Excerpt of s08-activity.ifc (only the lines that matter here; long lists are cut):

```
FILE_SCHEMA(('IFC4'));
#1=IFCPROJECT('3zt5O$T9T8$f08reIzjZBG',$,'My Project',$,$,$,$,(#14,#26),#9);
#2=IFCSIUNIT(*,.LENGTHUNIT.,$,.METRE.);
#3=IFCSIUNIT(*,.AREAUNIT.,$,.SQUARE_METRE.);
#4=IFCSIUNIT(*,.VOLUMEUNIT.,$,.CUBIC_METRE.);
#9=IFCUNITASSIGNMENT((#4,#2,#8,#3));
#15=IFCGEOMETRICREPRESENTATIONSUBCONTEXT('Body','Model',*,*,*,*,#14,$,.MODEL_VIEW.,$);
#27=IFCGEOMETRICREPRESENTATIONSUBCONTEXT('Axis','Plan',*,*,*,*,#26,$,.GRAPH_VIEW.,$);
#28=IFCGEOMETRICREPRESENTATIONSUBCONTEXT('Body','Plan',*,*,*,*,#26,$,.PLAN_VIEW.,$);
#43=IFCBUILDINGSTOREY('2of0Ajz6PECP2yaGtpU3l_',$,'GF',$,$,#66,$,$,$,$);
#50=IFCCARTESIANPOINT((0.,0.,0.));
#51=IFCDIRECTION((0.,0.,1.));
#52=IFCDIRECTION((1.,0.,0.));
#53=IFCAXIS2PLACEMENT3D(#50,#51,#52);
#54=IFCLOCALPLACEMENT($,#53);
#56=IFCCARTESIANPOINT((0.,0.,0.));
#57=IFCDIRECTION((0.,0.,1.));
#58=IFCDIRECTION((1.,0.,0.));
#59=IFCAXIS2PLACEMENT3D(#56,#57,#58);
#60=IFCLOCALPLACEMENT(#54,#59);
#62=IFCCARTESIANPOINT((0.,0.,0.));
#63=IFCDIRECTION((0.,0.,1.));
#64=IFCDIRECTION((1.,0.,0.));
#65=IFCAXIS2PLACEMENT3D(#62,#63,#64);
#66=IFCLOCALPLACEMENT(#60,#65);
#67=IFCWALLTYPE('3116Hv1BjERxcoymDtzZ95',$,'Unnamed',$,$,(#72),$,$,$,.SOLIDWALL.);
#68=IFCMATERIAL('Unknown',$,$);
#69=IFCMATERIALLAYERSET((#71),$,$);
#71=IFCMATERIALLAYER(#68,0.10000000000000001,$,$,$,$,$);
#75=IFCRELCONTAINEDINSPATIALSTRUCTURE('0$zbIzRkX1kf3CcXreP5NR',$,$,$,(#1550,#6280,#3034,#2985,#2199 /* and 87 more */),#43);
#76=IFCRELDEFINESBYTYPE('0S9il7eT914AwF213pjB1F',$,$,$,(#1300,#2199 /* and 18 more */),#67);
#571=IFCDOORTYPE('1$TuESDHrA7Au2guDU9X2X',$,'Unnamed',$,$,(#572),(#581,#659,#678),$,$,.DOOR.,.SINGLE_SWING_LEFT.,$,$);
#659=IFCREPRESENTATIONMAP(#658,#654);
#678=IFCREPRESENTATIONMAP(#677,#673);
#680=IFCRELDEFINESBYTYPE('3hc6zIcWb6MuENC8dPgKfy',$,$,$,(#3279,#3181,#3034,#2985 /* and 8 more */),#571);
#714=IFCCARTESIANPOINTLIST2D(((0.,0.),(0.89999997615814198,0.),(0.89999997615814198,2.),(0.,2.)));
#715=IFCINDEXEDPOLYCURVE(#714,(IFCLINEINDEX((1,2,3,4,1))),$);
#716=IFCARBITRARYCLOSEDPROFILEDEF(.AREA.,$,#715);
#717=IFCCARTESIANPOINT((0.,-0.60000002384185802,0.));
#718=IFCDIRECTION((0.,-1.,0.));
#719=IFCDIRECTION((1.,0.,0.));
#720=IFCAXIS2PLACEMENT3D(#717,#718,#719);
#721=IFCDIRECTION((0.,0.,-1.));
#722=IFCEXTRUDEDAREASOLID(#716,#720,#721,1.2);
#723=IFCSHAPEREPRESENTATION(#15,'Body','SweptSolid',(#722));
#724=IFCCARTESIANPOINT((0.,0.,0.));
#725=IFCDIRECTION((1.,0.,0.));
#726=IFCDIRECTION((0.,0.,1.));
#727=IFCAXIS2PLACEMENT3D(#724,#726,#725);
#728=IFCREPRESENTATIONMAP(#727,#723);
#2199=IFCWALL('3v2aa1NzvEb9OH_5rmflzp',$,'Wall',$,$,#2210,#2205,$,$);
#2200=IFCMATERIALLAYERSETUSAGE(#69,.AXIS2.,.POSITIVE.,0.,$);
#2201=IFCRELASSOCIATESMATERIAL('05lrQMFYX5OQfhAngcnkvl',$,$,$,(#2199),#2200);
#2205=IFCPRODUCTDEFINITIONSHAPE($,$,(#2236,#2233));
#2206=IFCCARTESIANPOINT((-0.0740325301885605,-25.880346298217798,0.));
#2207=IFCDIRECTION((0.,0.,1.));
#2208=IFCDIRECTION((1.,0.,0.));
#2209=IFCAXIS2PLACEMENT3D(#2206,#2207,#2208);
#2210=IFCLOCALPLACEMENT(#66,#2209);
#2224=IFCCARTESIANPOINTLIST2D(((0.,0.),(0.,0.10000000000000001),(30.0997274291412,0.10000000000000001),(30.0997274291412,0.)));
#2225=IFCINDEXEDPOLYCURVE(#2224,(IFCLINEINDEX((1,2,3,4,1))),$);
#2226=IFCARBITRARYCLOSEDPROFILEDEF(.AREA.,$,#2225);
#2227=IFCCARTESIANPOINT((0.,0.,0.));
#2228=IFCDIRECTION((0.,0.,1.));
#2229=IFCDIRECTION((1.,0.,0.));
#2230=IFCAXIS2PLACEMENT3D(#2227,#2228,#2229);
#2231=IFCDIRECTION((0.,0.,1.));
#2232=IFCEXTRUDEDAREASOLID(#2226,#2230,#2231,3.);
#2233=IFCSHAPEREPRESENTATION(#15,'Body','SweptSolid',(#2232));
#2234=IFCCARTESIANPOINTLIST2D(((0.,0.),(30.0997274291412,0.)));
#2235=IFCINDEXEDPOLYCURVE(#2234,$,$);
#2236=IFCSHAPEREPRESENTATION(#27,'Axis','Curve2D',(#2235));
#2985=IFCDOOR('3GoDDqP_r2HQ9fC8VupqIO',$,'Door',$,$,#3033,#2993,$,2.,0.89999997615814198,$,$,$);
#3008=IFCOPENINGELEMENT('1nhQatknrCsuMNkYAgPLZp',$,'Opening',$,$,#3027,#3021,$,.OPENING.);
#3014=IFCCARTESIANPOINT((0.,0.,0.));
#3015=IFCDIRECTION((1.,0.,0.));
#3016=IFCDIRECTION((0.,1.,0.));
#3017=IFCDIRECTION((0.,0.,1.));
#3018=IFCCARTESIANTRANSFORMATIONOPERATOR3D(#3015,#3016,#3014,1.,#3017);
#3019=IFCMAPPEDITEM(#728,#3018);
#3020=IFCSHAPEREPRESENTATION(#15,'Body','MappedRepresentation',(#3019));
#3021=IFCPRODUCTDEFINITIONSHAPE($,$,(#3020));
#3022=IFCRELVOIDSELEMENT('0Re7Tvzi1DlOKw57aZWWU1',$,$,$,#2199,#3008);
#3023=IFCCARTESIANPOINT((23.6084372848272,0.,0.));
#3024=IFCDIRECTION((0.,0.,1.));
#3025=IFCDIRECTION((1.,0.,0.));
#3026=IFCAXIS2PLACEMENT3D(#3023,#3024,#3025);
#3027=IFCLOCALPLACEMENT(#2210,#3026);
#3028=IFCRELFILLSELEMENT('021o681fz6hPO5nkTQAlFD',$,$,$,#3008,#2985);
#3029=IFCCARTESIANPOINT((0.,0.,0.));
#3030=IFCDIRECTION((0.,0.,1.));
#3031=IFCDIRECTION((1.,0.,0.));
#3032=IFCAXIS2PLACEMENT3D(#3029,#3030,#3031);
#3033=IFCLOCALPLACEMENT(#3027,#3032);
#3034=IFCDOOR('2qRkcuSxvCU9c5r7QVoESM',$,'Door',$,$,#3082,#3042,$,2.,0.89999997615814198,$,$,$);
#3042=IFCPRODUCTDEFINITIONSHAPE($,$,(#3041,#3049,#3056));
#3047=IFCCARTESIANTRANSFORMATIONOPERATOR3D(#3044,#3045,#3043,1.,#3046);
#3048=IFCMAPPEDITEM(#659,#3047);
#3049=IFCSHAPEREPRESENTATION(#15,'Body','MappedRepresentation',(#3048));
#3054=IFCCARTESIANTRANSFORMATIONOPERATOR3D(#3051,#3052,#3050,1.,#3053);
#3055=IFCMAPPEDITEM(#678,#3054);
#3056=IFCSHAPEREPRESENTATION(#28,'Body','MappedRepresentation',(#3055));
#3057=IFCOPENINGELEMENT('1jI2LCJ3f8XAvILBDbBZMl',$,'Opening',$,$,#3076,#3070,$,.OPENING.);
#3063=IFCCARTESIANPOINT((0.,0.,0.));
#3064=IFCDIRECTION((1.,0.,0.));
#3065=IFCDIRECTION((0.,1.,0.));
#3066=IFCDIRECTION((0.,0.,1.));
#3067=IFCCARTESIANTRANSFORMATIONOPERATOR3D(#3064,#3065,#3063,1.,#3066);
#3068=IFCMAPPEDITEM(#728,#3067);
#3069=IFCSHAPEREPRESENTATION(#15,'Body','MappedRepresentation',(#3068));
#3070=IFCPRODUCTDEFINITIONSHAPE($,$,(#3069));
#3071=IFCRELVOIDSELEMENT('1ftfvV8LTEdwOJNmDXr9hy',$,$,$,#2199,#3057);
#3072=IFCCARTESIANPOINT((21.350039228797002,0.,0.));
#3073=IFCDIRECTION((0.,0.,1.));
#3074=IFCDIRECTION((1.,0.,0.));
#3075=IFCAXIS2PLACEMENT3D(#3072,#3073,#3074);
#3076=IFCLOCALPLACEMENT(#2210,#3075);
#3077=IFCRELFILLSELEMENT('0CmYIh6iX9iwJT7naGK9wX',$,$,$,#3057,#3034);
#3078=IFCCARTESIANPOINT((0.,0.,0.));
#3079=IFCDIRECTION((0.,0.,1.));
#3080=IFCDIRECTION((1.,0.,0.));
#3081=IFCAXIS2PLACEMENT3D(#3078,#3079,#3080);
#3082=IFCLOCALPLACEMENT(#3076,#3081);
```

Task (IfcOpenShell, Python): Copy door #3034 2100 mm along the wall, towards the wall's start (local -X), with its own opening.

```python
import ifcopenshell
import ifcopenshell.api.feature
import ifcopenshell.api.geometry
import ifcopenshell.api.root
import ifcopenshell.geom
import ifcopenshell.util.element
import ifcopenshell.util.placement
import ifcopenshell.util.shape
import ifcopenshell.util.unit

model = ifcopenshell.open("s08-activity.ifc")
unit_scale = ifcopenshell.util.unit.calculate_unit_scale(model)
settings = ifcopenshell.geom.settings()


def volume(element):
    """Net volume in cubic metres, openings subtracted."""
    shape = ifcopenshell.geom.create_shape(settings, element)
    return ifcopenshell.util.shape.get_volume(shape.geometry)


door = model.by_guid("2qRkcuSxvCU9c5r7QVoESM")
opening = door.FillsVoids[0].RelatingOpeningElement
wall = opening.VoidsElements[0].RelatingBuildingElement
before = volume(wall)
shift = ifcopenshell.util.placement.get_local_placement(wall.ObjectPlacement)[:3, 0] * -2.1 / unit_scale

# copy_class copies the void relationship, type, container and properties, but no geometry.
new_opening = ifcopenshell.api.root.copy_class(model, product=opening)
new_opening.Representation = ifcopenshell.util.element.copy_deep(
    model, opening.Representation, exclude=["IfcGeometricRepresentationContext", "IfcRepresentationMap"]
)
new_door = ifcopenshell.api.root.copy_class(model, product=door)
new_door.Representation = ifcopenshell.util.element.copy_deep(
    model, door.Representation, exclude=["IfcGeometricRepresentationContext", "IfcRepresentationMap"]
)
ifcopenshell.api.feature.add_filling(model, opening=new_opening, element=new_door)

for old, new in ((opening, new_opening), (door, new_door)):
    matrix = ifcopenshell.util.placement.get_local_placement(old.ObjectPlacement)
    matrix[:3, 3] += shift
    ifcopenshell.api.geometry.edit_object_placement(model, product=new, matrix=matrix, is_si=False)

after = volume(wall)

print(f"wall volume {before:.3f} -> {after:.3f} m3")

model.write("s08-activity_rev.ifc")
```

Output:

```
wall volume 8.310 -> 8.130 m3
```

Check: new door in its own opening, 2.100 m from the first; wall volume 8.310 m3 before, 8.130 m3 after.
